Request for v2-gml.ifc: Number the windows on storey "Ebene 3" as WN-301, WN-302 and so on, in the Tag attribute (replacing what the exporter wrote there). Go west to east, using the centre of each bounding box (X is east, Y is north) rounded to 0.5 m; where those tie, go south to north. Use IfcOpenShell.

First a look at what the model holds.

```python
import ifcopenshell
import ifcopenshell.util.element
import ifcopenshell.util.placement

model = ifcopenshell.open("v2-gml.ifc")
print(model.schema)
storey = next(s for s in model.by_type("IfcBuildingStorey") if s.Name == "Ebene 3")
windows = [e for e in ifcopenshell.util.element.get_decomposition(storey) if e.is_a("IfcWindow")]
for e in sorted(windows, key=lambda e: e.id()):
    origin = ifcopenshell.util.placement.get_local_placement(e.ObjectPlacement)[:3, 3]
    print(e.id(), e.Tag, e.Name, origin.round(2) + 0.0, sep=" | ")
```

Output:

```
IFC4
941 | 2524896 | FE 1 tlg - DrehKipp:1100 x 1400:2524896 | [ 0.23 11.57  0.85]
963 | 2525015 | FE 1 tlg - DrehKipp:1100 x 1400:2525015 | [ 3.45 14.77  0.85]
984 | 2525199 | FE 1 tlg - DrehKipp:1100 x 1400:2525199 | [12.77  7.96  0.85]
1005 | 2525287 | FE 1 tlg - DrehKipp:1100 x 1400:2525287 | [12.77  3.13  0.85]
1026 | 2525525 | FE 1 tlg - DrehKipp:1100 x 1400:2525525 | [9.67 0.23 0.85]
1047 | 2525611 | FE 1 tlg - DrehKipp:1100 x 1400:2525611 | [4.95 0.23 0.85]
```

```python
import ifcopenshell
import ifcopenshell.geom
import ifcopenshell.util.element
import ifcopenshell.util.shape

model = ifcopenshell.open("v2-gml.ifc")
settings = ifcopenshell.geom.settings()
settings.set("use-world-coords", True)


def centre(element):
    shape = ifcopenshell.geom.create_shape(settings, element)
    return ifcopenshell.util.shape.get_bbox_centroid(shape.geometry)


storey = next(s for s in model.by_type("IfcBuildingStorey") if s.Name == "Ebene 3")
windows = [e for e in ifcopenshell.util.element.get_decomposition(storey) if e.is_a("IfcWindow")]

# Insertion points can sit at a corner or the storey origin, so sort by the geometry (in metres).
centres = {e: centre(e) for e in windows}
windows.sort(key=lambda e: (round(centres[e][0] / 0.5), centres[e][1]))

for i, e in enumerate(windows, start=1):
    number = f"WN-3{i:02d}"
    e.Tag = number
    print(e.id(), number)

model.write("v2-gml_edited.ifc")
```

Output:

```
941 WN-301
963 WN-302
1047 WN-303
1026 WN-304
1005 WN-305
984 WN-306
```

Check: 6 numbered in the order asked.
